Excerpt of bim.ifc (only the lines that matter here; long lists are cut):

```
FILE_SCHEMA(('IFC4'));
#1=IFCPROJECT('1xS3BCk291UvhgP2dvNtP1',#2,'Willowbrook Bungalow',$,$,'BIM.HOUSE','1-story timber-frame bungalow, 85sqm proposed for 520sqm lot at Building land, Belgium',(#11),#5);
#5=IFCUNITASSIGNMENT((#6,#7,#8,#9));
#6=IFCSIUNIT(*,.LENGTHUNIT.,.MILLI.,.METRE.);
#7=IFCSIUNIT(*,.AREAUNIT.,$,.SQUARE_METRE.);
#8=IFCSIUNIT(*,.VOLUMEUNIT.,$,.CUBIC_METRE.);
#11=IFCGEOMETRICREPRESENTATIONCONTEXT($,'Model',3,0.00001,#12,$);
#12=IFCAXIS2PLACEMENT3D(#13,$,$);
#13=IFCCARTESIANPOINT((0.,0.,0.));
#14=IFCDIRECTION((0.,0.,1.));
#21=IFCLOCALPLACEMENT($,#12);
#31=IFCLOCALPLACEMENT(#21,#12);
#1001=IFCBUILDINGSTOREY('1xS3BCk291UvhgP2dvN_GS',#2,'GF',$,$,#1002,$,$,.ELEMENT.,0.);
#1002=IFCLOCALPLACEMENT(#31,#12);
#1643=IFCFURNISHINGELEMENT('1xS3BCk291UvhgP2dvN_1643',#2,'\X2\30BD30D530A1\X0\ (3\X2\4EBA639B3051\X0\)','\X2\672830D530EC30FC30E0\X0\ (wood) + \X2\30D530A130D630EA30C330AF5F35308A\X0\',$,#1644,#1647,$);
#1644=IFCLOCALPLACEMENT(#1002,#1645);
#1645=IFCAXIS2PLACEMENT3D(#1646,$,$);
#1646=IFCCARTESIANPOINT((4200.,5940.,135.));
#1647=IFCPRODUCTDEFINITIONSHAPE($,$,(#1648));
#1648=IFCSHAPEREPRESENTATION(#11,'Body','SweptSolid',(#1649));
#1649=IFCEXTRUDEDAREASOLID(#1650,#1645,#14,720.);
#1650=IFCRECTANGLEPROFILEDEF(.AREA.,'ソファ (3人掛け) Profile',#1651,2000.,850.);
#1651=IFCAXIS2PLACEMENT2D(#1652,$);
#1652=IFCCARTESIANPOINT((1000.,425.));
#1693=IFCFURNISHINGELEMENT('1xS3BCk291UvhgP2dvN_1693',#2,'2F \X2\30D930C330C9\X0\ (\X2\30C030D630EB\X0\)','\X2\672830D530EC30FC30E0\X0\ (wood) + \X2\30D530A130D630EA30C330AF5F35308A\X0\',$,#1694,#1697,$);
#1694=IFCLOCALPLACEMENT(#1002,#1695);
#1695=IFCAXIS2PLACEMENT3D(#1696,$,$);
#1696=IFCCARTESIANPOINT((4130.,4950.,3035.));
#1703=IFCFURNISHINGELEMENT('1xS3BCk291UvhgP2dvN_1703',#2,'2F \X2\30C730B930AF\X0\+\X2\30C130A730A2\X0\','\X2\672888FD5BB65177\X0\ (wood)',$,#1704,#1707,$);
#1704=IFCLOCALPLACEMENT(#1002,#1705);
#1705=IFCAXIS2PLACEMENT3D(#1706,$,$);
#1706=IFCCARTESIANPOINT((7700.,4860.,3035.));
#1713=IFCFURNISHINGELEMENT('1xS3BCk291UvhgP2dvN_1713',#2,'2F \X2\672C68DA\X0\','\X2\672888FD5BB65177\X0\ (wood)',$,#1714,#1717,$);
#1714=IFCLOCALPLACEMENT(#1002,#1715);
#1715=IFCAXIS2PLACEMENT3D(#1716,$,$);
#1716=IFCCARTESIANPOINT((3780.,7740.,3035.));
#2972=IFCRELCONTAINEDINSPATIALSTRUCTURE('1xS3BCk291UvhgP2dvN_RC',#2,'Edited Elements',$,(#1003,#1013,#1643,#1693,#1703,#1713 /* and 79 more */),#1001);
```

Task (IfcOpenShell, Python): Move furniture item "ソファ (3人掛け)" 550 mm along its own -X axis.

```python
import ifcopenshell
import ifcopenshell.api.geometry
import ifcopenshell.util.placement

model = ifcopenshell.open("bim.ifc")

item = model.by_guid("1xS3BCk291UvhgP2dvN_1643")
matrix = ifcopenshell.util.placement.get_local_placement(item.ObjectPlacement)
matrix[:3, 3] -= matrix[:3, 0] * 550.0
ifcopenshell.api.geometry.edit_object_placement(model, product=item, matrix=matrix, is_si=False)

print(ifcopenshell.util.placement.get_local_placement(item.ObjectPlacement).round(3) + 0.0)

model.write("bim_edited.ifc")
```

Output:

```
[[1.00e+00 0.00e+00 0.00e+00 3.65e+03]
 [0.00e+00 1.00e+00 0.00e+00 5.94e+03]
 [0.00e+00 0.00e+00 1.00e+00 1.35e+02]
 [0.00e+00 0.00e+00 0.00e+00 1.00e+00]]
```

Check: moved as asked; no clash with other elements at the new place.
